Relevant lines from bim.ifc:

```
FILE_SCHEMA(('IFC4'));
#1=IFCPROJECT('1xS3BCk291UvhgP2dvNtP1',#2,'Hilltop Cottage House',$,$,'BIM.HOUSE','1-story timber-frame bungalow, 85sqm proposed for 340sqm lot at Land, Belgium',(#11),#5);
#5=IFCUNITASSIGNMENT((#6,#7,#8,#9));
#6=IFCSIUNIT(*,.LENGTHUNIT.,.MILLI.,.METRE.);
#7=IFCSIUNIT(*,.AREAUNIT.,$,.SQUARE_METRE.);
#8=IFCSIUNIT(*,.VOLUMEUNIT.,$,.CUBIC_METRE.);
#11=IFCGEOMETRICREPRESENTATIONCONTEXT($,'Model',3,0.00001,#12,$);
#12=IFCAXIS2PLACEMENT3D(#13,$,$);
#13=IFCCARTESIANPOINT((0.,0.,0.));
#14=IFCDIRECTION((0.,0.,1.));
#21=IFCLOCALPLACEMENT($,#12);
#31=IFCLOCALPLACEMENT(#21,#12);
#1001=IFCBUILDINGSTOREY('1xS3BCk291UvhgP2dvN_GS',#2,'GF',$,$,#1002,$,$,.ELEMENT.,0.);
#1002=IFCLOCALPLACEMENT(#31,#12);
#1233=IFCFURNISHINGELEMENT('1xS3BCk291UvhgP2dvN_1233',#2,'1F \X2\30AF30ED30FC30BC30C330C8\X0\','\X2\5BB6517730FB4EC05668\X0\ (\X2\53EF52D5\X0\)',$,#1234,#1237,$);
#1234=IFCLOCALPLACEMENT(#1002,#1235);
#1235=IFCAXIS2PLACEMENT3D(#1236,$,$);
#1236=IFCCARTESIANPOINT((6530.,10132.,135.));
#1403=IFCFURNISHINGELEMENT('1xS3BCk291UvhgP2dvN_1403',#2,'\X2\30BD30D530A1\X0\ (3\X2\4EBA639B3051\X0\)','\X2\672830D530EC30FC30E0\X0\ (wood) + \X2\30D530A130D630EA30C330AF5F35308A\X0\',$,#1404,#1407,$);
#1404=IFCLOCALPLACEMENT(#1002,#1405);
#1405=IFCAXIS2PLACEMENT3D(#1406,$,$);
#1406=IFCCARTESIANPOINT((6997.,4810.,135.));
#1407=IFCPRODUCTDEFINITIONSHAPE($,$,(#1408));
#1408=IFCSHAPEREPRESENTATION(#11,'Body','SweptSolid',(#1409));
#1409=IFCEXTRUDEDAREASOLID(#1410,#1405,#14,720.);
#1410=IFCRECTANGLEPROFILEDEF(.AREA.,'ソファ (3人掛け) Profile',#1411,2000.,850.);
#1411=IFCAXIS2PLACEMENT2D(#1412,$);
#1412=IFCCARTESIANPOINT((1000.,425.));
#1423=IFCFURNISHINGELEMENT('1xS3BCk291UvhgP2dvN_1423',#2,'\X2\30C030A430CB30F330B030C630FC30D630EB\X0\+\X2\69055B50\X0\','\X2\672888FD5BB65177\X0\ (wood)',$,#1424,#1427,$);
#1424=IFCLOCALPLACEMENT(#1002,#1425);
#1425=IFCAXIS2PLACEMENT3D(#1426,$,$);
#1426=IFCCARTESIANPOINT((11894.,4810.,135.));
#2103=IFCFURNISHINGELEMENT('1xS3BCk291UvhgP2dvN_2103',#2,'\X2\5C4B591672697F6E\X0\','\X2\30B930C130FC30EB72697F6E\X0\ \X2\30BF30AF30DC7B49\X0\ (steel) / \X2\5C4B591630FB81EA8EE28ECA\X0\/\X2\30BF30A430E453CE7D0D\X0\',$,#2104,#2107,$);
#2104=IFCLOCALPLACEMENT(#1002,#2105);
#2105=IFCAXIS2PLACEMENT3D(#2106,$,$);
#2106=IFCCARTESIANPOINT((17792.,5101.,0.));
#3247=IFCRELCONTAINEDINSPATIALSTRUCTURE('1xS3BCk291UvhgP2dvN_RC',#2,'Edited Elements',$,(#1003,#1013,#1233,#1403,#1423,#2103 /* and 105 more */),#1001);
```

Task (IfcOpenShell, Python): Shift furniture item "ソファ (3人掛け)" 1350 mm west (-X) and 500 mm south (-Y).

```python
import ifcopenshell
import ifcopenshell.api.geometry
import ifcopenshell.util.placement
import ifcopenshell.util.unit

model = ifcopenshell.open("bim.ifc")
unit_scale = ifcopenshell.util.unit.calculate_unit_scale(model)

item = model.by_guid("1xS3BCk291UvhgP2dvN_1403")
matrix = ifcopenshell.util.placement.get_local_placement(item.ObjectPlacement)
matrix[0, 3] -= 1.35 / unit_scale
matrix[1, 3] -= 0.5 / unit_scale
ifcopenshell.api.geometry.edit_object_placement(model, product=item, matrix=matrix, is_si=False)

print(ifcopenshell.util.placement.get_local_placement(item.ObjectPlacement).round(3) + 0.0)

model.write("bim_rev.ifc")
```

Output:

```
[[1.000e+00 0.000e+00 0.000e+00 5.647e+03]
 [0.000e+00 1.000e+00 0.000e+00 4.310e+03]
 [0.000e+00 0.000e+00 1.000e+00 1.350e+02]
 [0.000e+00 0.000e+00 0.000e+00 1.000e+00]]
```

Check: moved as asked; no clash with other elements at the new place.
